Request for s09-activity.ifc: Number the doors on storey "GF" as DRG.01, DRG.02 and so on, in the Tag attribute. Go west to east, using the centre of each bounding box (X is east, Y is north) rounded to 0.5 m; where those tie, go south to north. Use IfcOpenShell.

First a look at what the model holds.

```python
import ifcopenshell
import ifcopenshell.util.element
import ifcopenshell.util.placement

model = ifcopenshell.open("s09-activity.ifc")
print(model.schema)
storey = next(s for s in model.by_type("IfcBuildingStorey") if s.Name == "GF")
doors = [e for e in ifcopenshell.util.element.get_decomposition(storey) if e.is_a("IfcDoor")]
for e in sorted(doors, key=lambda e: e.id()):
    origin = ifcopenshell.util.placement.get_local_placement(e.ObjectPlacement)[:3, 3]
    print(e.id(), e.Tag, e.Name, origin.round(2) + 0.0, sep=" | ")
```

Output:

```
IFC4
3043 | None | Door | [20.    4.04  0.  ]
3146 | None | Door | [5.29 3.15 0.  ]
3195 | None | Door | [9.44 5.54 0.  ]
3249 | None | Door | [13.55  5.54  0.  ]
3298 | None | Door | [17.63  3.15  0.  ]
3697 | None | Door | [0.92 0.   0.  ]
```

```python
import ifcopenshell
import ifcopenshell.geom
import ifcopenshell.util.element
import ifcopenshell.util.shape

model = ifcopenshell.open("s09-activity.ifc")
settings = ifcopenshell.geom.settings()
settings.set("use-world-coords", True)


def centre(element):
    shape = ifcopenshell.geom.create_shape(settings, element)
    return ifcopenshell.util.shape.get_bbox_centroid(shape.geometry)


storey = next(s for s in model.by_type("IfcBuildingStorey") if s.Name == "GF")
doors = [e for e in ifcopenshell.util.element.get_decomposition(storey) if e.is_a("IfcDoor")]

# Insertion points can sit at a corner or the storey origin, so sort by the geometry (in metres).
centres = {e: centre(e) for e in doors}
doors.sort(key=lambda e: (round(centres[e][0] / 0.5), centres[e][1]))

for i, e in enumerate(doors, start=1):
    number = f"DRG.{i:02d}"
    e.Tag = number
    print(e.id(), number)

model.write("s09-activity_rev.ifc")
```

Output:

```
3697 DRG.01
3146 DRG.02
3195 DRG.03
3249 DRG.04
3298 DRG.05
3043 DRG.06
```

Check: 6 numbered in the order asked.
